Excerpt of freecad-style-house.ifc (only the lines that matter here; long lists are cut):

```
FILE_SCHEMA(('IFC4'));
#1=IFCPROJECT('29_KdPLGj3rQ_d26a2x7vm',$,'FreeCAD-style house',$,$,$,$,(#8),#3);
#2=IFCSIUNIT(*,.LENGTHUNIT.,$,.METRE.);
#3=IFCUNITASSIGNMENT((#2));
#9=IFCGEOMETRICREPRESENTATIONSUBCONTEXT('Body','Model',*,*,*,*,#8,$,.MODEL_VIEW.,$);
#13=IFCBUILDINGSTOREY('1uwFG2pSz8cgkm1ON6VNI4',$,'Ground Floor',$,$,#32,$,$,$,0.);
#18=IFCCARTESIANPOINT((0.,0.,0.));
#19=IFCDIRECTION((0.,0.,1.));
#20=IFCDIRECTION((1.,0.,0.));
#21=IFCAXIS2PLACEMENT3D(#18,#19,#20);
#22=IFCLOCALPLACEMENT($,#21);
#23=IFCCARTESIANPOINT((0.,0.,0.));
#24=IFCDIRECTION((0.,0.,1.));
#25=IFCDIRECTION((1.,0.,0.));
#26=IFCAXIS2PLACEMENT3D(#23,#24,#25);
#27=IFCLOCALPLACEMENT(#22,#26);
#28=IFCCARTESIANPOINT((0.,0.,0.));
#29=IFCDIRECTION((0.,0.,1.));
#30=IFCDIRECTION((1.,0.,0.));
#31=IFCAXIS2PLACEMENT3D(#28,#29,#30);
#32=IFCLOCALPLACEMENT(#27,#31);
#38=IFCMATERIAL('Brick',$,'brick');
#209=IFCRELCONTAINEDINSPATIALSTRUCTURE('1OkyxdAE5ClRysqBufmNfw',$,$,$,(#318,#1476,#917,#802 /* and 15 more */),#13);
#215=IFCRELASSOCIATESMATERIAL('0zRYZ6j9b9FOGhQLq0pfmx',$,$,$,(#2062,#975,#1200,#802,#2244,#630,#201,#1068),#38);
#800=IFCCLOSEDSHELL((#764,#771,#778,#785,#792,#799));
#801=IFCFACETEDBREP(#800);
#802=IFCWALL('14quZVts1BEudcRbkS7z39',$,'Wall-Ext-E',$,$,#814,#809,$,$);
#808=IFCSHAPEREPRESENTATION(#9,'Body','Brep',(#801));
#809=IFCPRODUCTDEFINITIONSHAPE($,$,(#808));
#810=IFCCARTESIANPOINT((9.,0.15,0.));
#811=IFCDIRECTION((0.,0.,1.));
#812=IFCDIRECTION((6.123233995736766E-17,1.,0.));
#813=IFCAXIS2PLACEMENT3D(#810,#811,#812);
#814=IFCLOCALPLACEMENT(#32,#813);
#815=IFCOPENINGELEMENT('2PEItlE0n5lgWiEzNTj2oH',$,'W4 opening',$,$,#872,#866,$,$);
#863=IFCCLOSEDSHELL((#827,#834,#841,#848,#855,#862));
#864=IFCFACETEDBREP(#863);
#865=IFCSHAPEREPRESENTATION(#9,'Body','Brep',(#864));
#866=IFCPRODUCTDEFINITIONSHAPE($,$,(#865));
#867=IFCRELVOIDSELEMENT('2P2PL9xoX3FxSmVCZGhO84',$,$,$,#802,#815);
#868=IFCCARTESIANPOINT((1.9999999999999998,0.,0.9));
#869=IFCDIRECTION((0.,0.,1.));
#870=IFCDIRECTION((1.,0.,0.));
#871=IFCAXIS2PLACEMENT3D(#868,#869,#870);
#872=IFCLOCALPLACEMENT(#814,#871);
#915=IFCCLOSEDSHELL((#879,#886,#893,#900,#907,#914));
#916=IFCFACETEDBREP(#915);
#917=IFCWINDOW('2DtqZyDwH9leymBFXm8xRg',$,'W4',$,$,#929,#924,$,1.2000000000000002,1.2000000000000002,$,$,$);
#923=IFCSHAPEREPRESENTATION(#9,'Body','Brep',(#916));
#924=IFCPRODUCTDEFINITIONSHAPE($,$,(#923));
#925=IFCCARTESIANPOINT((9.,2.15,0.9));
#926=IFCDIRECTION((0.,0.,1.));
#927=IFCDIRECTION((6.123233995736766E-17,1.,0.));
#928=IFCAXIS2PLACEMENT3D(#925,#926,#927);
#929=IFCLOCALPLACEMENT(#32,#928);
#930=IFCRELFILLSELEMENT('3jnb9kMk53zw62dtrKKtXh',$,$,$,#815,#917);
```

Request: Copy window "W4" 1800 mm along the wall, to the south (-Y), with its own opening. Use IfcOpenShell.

```python
import ifcopenshell
import ifcopenshell.api.feature
import ifcopenshell.api.geometry
import ifcopenshell.api.root
import ifcopenshell.geom
import ifcopenshell.util.element
import ifcopenshell.util.placement
import ifcopenshell.util.shape

model = ifcopenshell.open("freecad-style-house.ifc")
settings = ifcopenshell.geom.settings()


def volume(element):
    """Net volume in cubic metres, openings subtracted."""
    shape = ifcopenshell.geom.create_shape(settings, element)
    return ifcopenshell.util.shape.get_volume(shape.geometry)


window = model.by_guid("2DtqZyDwH9leymBFXm8xRg")
opening = window.FillsVoids[0].RelatingOpeningElement
wall = opening.VoidsElements[0].RelatingBuildingElement
before = volume(wall)
shift = ifcopenshell.util.placement.get_local_placement(wall.ObjectPlacement)[:3, 0] * -1.8

# copy_class copies the void relationship, type, container and properties, but no geometry.
new_opening = ifcopenshell.api.root.copy_class(model, product=opening)
new_opening.Representation = ifcopenshell.util.element.copy_deep(
    model, opening.Representation, exclude=["IfcGeometricRepresentationContext", "IfcRepresentationMap"]
)
new_window = ifcopenshell.api.root.copy_class(model, product=window)
new_window.Representation = ifcopenshell.util.element.copy_deep(
    model, window.Representation, exclude=["IfcGeometricRepresentationContext", "IfcRepresentationMap"]
)
ifcopenshell.api.feature.add_filling(model, opening=new_opening, element=new_window)

for old, new in ((opening, new_opening), (window, new_window)):
    matrix = ifcopenshell.util.placement.get_local_placement(old.ObjectPlacement)
    matrix[:3, 3] += shift
    ifcopenshell.api.geometry.edit_object_placement(model, product=new, matrix=matrix, is_si=False)

after = volume(wall)

print(f"wall volume {before:.3f} -> {after:.3f} m3")

model.write("freecad-style-house_updated.ifc")
```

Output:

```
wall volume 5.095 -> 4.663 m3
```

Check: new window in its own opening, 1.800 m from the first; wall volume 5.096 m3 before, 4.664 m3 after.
